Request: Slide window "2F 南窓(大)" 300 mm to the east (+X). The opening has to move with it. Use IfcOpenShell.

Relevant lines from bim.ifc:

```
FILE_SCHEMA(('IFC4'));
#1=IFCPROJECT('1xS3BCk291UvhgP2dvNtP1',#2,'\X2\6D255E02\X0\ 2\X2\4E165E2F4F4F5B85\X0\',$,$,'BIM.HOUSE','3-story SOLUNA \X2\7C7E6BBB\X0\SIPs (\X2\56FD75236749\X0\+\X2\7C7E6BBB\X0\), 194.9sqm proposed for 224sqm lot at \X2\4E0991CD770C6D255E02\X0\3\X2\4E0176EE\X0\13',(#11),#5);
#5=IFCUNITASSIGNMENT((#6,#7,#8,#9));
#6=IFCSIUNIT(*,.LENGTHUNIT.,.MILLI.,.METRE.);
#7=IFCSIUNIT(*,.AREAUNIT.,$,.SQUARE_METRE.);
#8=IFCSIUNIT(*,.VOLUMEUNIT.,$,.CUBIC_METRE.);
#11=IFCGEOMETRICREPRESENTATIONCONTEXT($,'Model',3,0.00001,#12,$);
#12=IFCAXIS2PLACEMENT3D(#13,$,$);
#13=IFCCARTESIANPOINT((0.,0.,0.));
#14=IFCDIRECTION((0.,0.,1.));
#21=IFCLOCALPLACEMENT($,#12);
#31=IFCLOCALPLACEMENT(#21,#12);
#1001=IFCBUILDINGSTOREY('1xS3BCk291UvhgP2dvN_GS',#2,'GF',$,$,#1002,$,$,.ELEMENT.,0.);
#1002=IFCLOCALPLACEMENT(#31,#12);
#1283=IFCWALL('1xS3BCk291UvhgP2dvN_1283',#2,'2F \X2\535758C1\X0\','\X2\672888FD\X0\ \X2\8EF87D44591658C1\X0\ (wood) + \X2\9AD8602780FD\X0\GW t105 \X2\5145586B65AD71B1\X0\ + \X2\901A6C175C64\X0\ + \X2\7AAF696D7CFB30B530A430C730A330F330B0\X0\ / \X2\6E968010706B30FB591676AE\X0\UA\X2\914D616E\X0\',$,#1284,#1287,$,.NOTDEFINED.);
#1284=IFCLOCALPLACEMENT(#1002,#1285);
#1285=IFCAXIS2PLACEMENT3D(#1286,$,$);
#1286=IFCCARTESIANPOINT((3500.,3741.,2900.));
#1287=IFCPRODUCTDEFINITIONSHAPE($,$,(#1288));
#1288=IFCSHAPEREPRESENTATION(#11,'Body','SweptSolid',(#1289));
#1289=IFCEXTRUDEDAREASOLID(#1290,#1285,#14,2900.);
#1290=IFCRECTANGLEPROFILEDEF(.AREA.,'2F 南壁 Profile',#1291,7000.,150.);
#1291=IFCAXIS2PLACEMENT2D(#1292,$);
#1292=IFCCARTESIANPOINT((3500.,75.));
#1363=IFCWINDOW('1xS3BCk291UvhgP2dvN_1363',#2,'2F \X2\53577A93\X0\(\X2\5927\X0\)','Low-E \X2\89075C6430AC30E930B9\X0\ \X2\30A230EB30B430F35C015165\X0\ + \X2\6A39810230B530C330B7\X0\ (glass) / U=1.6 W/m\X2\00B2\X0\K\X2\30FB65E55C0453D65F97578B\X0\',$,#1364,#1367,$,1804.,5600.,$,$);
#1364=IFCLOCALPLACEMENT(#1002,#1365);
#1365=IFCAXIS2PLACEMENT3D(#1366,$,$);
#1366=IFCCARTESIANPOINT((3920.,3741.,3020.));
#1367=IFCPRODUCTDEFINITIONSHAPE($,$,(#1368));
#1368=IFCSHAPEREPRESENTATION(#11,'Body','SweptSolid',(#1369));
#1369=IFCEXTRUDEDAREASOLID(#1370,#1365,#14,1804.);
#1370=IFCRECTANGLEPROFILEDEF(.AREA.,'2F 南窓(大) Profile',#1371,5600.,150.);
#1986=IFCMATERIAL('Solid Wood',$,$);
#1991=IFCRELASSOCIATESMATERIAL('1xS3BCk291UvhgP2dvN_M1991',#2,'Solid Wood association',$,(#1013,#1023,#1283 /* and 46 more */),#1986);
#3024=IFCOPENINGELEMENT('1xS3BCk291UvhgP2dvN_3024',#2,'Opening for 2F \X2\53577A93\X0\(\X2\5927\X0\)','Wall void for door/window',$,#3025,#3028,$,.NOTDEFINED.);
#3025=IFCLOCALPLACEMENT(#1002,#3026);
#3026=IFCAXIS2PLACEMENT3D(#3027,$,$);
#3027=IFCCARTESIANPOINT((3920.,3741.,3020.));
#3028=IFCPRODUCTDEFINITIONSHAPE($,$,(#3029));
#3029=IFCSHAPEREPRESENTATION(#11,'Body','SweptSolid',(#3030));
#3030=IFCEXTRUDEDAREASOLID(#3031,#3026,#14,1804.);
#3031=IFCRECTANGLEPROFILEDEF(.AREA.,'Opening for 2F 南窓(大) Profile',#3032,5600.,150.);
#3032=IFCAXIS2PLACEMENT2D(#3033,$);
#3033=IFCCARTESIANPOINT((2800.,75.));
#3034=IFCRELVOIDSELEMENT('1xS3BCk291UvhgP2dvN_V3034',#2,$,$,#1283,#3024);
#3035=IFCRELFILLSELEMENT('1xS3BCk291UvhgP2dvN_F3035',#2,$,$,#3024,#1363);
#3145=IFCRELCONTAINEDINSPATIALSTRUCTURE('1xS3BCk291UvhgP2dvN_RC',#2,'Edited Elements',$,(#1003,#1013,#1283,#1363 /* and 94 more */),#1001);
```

```python
import ifcopenshell
import ifcopenshell.api.geometry
import ifcopenshell.util.placement
import ifcopenshell.util.unit

model = ifcopenshell.open("bim.ifc")
unit_scale = ifcopenshell.util.unit.calculate_unit_scale(model)

window = model.by_guid("1xS3BCk291UvhgP2dvN_1363")
opening = window.FillsVoids[0].RelatingOpeningElement
wall = opening.VoidsElements[0].RelatingBuildingElement

wall_matrix = ifcopenshell.util.placement.get_local_placement(wall.ObjectPlacement)
shift = wall_matrix[:3, 0] * 0.3 / unit_scale
before = ifcopenshell.util.placement.get_local_placement(window.ObjectPlacement)[:3, 3].copy()

# The window is not placed relative to its opening, so move both.
for product in (opening, window):
    matrix = ifcopenshell.util.placement.get_local_placement(product.ObjectPlacement)
    matrix[:3, 3] += shift
    ifcopenshell.api.geometry.edit_object_placement(model, product=product, matrix=matrix, is_si=False)

after = ifcopenshell.util.placement.get_local_placement(window.ObjectPlacement)[:3, 3]
print("window moved by", (after - before).round(3) + 0.0)

model.write("bim-out.ifc")
```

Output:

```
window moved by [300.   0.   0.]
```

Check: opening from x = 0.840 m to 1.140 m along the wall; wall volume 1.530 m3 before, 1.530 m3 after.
